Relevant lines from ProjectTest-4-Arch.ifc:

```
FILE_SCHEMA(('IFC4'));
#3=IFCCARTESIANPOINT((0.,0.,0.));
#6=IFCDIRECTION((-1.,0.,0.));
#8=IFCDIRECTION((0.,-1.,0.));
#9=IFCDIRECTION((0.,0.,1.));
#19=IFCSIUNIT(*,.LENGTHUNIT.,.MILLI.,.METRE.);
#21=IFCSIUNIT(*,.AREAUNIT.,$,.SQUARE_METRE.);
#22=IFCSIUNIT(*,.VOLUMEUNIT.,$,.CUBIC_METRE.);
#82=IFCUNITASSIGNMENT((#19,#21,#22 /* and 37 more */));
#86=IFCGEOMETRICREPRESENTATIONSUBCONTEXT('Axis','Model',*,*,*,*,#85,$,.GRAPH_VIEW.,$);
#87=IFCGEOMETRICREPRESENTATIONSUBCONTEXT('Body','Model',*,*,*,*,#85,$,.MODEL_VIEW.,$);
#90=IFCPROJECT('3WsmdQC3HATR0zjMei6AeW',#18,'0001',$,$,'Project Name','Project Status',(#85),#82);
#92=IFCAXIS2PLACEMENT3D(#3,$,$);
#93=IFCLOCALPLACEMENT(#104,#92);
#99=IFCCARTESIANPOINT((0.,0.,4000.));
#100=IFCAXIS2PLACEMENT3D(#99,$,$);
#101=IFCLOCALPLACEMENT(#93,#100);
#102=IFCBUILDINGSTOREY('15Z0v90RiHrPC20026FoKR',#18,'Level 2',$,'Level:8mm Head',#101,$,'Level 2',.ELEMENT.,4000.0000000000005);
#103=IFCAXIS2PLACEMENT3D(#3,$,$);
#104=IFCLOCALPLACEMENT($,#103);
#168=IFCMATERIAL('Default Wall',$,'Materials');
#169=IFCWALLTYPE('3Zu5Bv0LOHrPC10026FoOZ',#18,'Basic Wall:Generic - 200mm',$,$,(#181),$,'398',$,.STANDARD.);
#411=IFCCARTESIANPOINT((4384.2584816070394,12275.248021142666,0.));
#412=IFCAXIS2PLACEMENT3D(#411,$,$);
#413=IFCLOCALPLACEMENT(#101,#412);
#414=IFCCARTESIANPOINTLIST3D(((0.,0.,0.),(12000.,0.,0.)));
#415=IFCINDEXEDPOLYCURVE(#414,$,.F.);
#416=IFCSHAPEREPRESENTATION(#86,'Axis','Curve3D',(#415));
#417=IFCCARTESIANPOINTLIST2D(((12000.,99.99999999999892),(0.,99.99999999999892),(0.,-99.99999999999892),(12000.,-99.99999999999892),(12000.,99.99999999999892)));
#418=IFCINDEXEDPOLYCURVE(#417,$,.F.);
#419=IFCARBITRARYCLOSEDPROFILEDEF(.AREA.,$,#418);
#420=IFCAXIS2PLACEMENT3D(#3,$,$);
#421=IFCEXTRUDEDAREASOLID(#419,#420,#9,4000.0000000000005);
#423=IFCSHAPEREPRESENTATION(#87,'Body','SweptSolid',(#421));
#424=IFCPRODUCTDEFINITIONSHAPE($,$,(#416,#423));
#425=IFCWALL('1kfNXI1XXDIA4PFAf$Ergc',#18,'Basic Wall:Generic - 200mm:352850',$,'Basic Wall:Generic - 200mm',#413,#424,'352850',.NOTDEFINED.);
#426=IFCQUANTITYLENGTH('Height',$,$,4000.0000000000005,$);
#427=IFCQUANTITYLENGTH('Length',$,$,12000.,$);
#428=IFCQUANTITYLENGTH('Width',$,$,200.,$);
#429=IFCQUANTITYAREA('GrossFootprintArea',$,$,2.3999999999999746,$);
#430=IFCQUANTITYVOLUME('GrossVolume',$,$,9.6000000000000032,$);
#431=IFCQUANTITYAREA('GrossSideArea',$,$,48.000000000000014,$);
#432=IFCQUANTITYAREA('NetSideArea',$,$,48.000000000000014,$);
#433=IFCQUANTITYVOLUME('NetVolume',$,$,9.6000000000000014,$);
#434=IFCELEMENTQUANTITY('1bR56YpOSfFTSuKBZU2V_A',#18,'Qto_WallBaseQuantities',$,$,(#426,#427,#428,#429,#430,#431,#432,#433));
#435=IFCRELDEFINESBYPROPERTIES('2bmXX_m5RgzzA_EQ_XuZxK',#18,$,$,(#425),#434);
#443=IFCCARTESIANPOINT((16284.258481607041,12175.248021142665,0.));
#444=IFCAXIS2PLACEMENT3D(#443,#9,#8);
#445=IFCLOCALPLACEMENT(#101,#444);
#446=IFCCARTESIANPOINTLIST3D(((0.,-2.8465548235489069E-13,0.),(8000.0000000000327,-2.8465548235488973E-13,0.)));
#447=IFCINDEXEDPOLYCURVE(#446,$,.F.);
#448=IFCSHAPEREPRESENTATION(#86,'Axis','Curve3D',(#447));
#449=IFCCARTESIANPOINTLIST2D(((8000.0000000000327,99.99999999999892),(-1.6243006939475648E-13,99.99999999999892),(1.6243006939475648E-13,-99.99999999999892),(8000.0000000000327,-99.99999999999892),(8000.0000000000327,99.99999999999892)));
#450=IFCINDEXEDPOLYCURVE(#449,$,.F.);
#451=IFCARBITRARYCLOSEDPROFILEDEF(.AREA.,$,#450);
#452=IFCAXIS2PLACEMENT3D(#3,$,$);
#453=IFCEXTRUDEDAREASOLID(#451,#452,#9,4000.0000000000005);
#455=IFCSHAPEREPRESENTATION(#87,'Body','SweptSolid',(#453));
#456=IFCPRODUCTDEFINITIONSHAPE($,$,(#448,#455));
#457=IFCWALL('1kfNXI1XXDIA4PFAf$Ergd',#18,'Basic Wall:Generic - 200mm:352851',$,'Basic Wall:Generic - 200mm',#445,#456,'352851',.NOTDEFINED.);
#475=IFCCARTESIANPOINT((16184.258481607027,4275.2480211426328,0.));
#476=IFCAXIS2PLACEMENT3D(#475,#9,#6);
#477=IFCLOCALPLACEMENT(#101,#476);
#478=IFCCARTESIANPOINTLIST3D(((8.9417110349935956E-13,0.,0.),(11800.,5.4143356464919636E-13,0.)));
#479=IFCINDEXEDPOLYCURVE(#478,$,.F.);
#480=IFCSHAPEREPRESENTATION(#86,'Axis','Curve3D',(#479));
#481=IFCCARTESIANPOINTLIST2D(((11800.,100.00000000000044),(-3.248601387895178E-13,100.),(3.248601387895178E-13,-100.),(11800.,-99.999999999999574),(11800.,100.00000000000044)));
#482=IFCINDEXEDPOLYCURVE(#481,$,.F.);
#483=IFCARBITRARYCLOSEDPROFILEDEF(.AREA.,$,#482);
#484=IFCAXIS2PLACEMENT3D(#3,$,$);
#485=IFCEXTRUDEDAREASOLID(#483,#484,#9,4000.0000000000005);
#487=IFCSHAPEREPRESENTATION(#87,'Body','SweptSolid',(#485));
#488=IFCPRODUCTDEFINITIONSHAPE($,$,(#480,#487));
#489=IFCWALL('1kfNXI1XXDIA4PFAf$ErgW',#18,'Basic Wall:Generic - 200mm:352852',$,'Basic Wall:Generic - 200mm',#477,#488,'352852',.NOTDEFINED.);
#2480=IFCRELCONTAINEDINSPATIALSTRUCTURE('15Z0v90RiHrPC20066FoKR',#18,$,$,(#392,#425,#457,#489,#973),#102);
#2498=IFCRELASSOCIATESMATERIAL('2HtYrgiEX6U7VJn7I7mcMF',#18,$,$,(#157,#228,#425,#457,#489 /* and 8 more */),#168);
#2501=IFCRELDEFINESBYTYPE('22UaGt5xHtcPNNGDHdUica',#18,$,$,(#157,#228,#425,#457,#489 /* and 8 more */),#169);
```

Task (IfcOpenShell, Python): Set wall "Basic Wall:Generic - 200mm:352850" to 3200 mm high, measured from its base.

```python
import ifcopenshell
import ifcopenshell.api.pset
import ifcopenshell.geom
import ifcopenshell.util.element
import ifcopenshell.util.representation
import ifcopenshell.util.shape
import ifcopenshell.util.unit

model = ifcopenshell.open("ProjectTest-4-Arch.ifc")
unit_scale = ifcopenshell.util.unit.calculate_unit_scale(model)
area_scale = ifcopenshell.util.unit.calculate_unit_scale(model, "AREAUNIT")
volume_scale = ifcopenshell.util.unit.calculate_unit_scale(model, "VOLUMEUNIT")
settings = ifcopenshell.geom.settings()


def volume(element):
    """Net volume in cubic metres, openings subtracted."""
    shape = ifcopenshell.geom.create_shape(settings, element)
    return ifcopenshell.util.shape.get_volume(shape.geometry)


wall = model.by_id(425)
before = volume(wall)

body = ifcopenshell.util.representation.get_representation(wall, "Model", "Body")
solid = body.Items[0]
old_height = solid.Depth
solid.Depth = 3.2 / unit_scale
after = volume(wall)
thickness = 0.2  # wall thickness in metres

# Update the stored height, areas and volumes.
qto = model.by_id(ifcopenshell.util.element.get_pset(wall, "Qto_WallBaseQuantities", should_inherit=False)["id"])
ifcopenshell.api.pset.edit_qto(model, qto=qto, properties={
    "Height": solid.Depth,
    "GrossVolume": ifcopenshell.util.element.get_pset(wall, "Qto_WallBaseQuantities", "GrossVolume") * solid.Depth / old_height,
    "GrossSideArea": ifcopenshell.util.element.get_pset(wall, "Qto_WallBaseQuantities", "GrossSideArea") * solid.Depth / old_height,
    "NetSideArea": after / thickness / area_scale,
    "NetVolume": after / volume_scale,
})

print(f"height {old_height:g} -> {solid.Depth:g}, volume {before:.3f} -> {after:.3f} m3")

model.write("ProjectTest-4-Arch-out.ifc")
```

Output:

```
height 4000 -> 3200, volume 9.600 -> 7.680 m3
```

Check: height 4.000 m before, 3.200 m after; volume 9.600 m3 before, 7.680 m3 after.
